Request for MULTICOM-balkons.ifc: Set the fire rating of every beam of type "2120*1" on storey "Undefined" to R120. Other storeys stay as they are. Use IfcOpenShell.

First a look at what the model holds.

```python
import ifcopenshell
import ifcopenshell.util.element

model = ifcopenshell.open("MULTICOM-balkons.ifc")
print(model.schema)
storey = next(s for s in model.by_type("IfcBuildingStorey") if s.Name == "Undefined")
beams = [e for e in ifcopenshell.util.element.get_decomposition(storey) if e.is_a("IfcBeam")]
seen = {}
for e in beams:
    element_type = ifcopenshell.util.element.get_type(e)
    key = (element_type.Name if element_type != e and element_type else None, ifcopenshell.util.element.get_pset(e, "Pset_BeamCommon", "FireRating"))
    seen[key] = seen.get(key, 0) + 1
for (name, value), count in sorted(seen.items(), key=str):
    print(count, "x", name, "|", value)
```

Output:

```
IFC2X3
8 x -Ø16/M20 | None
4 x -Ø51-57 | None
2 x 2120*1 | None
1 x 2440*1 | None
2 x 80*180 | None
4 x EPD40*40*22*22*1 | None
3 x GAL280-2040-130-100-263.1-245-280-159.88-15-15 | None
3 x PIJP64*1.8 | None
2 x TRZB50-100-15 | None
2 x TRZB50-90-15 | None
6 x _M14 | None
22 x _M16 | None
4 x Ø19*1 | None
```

```python
import ifcopenshell
import ifcopenshell.api.pset
import ifcopenshell.util.element

model = ifcopenshell.open("MULTICOM-balkons.ifc")

storey = next(s for s in model.by_type("IfcBuildingStorey") if s.Name == "Undefined")
beams = [e for e in ifcopenshell.util.element.get_decomposition(storey) if e.is_a("IfcBeam")]

count = 0
for e in beams:
    element_type = ifcopenshell.util.element.get_type(e)
    if element_type in (None, e) or element_type.Name != "2120*1":
        continue
    # add_pset returns the element's existing set when there is one.
    pset = ifcopenshell.api.pset.add_pset(model, product=e, name="Pset_BeamCommon")
    ifcopenshell.api.pset.edit_pset(model, pset=pset, properties={"FireRating": "R120"})
    count += 1

print(count, "beams updated")

model.write("MULTICOM-balkons_updated.ifc")
```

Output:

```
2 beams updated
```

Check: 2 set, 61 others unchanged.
